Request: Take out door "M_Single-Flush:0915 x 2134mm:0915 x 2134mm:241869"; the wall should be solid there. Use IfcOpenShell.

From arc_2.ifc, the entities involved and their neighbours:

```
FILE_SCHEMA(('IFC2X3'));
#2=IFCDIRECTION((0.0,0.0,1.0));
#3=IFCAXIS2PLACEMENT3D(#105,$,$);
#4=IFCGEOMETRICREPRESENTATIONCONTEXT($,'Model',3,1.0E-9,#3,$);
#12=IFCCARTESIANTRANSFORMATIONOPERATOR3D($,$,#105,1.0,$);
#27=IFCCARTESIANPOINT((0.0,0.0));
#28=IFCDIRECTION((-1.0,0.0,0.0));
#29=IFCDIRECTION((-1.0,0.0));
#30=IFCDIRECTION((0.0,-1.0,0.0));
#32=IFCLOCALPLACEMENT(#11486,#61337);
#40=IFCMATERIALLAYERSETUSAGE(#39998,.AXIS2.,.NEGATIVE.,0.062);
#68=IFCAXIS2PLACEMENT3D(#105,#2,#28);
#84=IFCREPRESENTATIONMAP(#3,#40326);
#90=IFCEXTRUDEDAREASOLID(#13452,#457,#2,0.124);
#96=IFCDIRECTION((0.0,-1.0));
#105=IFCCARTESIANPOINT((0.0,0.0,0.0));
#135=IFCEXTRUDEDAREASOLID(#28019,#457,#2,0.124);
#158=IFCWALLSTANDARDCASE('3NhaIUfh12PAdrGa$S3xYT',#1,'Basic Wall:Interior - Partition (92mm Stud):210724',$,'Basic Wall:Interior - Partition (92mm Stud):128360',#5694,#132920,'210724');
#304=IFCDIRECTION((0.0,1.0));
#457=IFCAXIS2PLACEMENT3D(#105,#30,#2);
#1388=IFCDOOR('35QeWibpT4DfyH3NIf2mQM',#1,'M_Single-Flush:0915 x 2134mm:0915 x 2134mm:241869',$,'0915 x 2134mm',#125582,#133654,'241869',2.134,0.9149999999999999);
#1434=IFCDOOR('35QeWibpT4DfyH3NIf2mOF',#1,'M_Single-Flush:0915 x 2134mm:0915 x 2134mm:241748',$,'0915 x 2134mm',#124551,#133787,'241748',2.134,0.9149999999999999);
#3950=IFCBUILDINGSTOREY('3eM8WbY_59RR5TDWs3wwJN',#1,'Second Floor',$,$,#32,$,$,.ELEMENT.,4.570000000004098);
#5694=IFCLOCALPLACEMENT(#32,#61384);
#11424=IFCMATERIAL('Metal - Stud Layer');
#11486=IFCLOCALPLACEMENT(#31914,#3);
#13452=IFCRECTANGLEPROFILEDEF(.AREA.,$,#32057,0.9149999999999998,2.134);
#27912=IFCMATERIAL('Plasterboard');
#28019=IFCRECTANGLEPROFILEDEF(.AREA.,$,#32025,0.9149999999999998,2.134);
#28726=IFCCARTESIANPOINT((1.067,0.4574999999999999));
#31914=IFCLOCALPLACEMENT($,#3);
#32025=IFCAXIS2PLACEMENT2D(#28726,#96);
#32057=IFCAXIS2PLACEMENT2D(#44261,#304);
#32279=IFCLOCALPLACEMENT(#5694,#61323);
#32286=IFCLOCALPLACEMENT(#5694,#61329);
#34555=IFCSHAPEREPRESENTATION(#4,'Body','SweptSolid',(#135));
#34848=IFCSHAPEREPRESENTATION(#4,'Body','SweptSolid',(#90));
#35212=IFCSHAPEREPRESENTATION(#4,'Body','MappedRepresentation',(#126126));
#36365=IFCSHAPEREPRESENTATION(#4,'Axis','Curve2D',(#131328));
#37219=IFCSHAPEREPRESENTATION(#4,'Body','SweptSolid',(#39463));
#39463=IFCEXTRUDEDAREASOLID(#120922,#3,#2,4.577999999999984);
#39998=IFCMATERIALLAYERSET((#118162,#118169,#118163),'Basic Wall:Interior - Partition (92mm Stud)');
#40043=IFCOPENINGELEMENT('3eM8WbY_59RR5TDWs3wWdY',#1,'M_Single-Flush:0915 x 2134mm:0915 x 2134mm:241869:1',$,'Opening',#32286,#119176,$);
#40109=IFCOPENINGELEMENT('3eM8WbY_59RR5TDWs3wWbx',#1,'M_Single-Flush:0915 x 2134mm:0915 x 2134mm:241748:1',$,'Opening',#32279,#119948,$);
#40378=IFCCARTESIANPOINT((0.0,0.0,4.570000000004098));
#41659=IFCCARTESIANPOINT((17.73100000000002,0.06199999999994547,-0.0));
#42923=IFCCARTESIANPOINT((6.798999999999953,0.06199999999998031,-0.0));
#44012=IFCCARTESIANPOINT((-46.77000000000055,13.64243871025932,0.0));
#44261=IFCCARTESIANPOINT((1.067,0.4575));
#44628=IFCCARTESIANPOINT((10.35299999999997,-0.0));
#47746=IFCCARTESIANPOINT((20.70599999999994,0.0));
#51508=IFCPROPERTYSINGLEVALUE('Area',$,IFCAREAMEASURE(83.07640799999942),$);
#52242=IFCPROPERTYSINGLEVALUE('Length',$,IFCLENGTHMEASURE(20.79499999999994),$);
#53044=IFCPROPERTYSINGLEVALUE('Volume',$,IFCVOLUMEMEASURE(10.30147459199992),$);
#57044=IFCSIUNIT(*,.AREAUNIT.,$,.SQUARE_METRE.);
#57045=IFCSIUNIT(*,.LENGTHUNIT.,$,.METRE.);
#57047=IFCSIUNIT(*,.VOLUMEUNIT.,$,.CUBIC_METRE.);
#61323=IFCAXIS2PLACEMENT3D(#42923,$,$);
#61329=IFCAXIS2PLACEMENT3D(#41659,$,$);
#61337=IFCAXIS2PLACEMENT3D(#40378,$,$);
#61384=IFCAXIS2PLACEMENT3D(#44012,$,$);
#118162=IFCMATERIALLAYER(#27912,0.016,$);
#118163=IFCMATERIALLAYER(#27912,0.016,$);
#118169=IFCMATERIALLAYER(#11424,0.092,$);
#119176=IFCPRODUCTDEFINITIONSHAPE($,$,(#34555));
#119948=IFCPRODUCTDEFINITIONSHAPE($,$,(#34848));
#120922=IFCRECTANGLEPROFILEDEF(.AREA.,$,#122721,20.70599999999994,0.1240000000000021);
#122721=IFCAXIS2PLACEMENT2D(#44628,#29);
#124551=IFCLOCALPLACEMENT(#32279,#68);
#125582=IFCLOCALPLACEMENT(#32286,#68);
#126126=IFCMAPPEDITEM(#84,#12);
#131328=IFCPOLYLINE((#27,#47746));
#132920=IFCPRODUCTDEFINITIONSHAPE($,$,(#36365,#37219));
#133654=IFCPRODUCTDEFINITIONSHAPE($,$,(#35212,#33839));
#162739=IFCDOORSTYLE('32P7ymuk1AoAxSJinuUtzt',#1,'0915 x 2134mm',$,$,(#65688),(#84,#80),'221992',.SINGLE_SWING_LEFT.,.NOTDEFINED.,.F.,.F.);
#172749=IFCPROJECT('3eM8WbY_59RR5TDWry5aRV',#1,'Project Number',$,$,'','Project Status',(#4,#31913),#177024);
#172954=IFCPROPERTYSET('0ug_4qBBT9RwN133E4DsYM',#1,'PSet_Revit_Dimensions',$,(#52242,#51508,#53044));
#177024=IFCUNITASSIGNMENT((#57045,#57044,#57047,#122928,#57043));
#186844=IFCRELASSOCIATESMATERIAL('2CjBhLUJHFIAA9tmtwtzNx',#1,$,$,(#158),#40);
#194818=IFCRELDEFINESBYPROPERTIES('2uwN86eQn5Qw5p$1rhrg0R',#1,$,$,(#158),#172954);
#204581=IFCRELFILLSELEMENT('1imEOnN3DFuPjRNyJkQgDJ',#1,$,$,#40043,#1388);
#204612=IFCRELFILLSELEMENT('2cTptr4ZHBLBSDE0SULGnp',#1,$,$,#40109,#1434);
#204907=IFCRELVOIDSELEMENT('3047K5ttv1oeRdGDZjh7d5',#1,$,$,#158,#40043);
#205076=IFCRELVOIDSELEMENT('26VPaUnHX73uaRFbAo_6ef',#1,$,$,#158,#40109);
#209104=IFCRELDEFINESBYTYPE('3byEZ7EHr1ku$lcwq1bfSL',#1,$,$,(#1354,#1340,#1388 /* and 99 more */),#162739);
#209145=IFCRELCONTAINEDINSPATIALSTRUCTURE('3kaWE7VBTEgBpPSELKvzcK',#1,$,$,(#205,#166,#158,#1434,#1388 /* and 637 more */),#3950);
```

```python
import ifcopenshell
import ifcopenshell.api.feature
import ifcopenshell.api.pset
import ifcopenshell.api.root
import ifcopenshell.geom
import ifcopenshell.util.element
import ifcopenshell.util.shape
import ifcopenshell.util.unit

model = ifcopenshell.open("arc_2.ifc")
area_scale = ifcopenshell.util.unit.calculate_unit_scale(model, "AREAUNIT")
volume_scale = ifcopenshell.util.unit.calculate_unit_scale(model, "VOLUMEUNIT")
settings = ifcopenshell.geom.settings()


def volume(element):
    """Net volume in cubic metres, openings subtracted."""
    shape = ifcopenshell.geom.create_shape(settings, element)
    return ifcopenshell.util.shape.get_volume(shape.geometry)


door = model.by_guid("35QeWibpT4DfyH3NIf2mQM")
opening = door.FillsVoids[0].RelatingOpeningElement
wall = opening.VoidsElements[0].RelatingBuildingElement
before = volume(wall)

ifcopenshell.api.root.remove_product(model, product=door)
ifcopenshell.api.feature.remove_feature(model, feature=opening)

after = volume(wall)
thickness = 0.124  # wall thickness in metres

# Update the wall's stored quantities.
pset = model.by_id(ifcopenshell.util.element.get_pset(wall, "PSet_Revit_Dimensions", should_inherit=False)["id"])
ifcopenshell.api.pset.edit_pset(model, pset=pset, properties={
    "Area": model.create_entity("IfcAreaMeasure", after / thickness / area_scale),
    "Volume": model.create_entity("IfcVolumeMeasure", after / volume_scale),
})

print(f"wall volume {before:.3f} -> {after:.3f} m3")

model.write("arc_2_v2.ifc")
```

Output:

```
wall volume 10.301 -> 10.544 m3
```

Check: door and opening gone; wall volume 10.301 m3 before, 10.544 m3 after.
